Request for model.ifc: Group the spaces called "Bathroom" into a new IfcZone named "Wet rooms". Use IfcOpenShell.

First a look at what the model holds.

```python
import ifcopenshell

model = ifcopenshell.open("model.ifc")
print(model.schema)
seen = {}
for space in model.by_type("IfcSpace"):
    seen[space.LongName] = seen.get(space.LongName, 0) + 1
for name, count in sorted(seen.items(), key=str):
    print(count, "x", name)
print("zones:", [z.Name for z in model.by_type("IfcZone")][:20])
```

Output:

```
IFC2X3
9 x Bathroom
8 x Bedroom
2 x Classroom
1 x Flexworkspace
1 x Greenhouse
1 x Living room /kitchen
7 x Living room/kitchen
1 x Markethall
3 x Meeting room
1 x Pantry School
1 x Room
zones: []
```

```python
import ifcopenshell
import ifcopenshell.api.group
import ifcopenshell.api.root

model = ifcopenshell.open("model.ifc")

names = {"Bathroom"}
spaces = [s for s in model.by_type("IfcSpace") if s.LongName in names]

zone = ifcopenshell.api.root.create_entity(model, ifc_class="IfcZone", name="Wet rooms")
ifcopenshell.api.group.assign_group(model, products=spaces, group=zone)
print(len(spaces), "spaces in", zone.Name)

model.write("model_rev.ifc")
```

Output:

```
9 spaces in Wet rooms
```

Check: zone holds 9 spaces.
